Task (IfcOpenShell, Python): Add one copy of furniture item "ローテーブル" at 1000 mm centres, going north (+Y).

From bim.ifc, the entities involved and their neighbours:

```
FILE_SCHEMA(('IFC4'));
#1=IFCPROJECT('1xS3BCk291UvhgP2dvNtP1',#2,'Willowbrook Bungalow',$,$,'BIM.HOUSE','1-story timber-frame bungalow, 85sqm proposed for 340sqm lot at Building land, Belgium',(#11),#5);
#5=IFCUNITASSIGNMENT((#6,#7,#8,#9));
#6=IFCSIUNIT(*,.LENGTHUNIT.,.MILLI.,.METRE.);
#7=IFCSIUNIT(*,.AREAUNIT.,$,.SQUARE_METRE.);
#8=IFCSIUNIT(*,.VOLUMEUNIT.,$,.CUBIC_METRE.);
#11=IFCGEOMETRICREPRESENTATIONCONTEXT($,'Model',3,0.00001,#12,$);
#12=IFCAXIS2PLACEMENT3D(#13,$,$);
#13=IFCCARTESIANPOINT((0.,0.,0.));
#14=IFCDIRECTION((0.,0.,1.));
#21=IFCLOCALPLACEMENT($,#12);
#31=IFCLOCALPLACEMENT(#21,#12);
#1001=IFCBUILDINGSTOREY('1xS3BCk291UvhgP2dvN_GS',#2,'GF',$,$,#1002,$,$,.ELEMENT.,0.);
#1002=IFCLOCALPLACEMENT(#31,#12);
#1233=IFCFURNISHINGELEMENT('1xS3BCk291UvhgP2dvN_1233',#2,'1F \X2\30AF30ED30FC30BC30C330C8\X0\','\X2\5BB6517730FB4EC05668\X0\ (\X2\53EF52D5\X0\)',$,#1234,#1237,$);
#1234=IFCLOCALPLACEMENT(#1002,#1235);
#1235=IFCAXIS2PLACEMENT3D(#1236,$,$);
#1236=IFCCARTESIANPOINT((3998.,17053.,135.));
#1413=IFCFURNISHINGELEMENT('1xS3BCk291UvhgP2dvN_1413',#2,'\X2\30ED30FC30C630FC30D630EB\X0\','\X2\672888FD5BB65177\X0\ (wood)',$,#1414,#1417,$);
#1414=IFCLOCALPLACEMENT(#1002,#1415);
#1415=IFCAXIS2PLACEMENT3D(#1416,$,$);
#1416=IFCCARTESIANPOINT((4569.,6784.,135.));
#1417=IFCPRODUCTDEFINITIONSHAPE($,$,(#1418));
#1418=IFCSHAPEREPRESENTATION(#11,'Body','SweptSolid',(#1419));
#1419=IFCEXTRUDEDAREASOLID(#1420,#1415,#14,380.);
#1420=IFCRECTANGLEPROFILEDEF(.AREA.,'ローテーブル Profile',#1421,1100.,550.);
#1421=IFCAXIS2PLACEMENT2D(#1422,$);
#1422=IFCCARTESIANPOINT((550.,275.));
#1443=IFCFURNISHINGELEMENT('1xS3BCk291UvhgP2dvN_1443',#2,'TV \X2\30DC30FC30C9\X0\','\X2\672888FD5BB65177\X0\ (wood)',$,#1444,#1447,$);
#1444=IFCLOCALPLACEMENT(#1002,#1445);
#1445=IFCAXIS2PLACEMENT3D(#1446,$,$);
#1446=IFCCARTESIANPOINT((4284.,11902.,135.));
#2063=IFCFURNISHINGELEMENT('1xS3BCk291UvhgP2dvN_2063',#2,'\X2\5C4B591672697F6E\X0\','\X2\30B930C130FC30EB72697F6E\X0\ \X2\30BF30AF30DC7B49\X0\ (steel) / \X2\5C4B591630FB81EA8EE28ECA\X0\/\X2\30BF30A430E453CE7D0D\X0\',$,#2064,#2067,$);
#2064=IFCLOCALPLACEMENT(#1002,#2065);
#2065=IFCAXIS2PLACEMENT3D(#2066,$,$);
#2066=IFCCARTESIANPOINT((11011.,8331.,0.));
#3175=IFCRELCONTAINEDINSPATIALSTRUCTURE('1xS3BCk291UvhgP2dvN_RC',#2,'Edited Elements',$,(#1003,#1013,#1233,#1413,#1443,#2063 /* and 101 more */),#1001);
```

```python
import numpy as np
import ifcopenshell
import ifcopenshell.api.geometry
import ifcopenshell.api.root
import ifcopenshell.util.element
import ifcopenshell.util.placement

model = ifcopenshell.open("bim.ifc")


def reuse_history(source, copy):
    """copy_class also copies each property set's owner history, people and application; keep the originals."""
    for rel in copy.IsDefinedBy:
        if rel.is_a("IfcRelDefinesByProperties") and (history := rel.RelatingPropertyDefinition.OwnerHistory):
            rel.RelatingPropertyDefinition.OwnerHistory = source.OwnerHistory
            ifcopenshell.util.element.remove_deep2(model, history)


source = model.by_guid("1xS3BCk291UvhgP2dvN_1413")
base = ifcopenshell.util.placement.get_local_placement(source.ObjectPlacement)
step = np.array([0.0, 1.0, 0.0]) * 1000.0

for i in range(1, 2):
    copy = ifcopenshell.api.root.copy_class(model, product=source)
    copy.Representation = ifcopenshell.util.element.copy_deep(
        model, source.Representation, exclude=["IfcGeometricRepresentationContext", "IfcRepresentationMap"]
    )
    reuse_history(source, copy)
    matrix = base.copy()
    matrix[:3, 3] += i * step
    print("added at", matrix[:3, 3].round(3) + 0.0)
    ifcopenshell.api.geometry.edit_object_placement(model, product=copy, matrix=matrix, is_si=False)

model.write("bim_updated.ifc")
```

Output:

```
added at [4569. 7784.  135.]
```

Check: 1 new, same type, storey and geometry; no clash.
